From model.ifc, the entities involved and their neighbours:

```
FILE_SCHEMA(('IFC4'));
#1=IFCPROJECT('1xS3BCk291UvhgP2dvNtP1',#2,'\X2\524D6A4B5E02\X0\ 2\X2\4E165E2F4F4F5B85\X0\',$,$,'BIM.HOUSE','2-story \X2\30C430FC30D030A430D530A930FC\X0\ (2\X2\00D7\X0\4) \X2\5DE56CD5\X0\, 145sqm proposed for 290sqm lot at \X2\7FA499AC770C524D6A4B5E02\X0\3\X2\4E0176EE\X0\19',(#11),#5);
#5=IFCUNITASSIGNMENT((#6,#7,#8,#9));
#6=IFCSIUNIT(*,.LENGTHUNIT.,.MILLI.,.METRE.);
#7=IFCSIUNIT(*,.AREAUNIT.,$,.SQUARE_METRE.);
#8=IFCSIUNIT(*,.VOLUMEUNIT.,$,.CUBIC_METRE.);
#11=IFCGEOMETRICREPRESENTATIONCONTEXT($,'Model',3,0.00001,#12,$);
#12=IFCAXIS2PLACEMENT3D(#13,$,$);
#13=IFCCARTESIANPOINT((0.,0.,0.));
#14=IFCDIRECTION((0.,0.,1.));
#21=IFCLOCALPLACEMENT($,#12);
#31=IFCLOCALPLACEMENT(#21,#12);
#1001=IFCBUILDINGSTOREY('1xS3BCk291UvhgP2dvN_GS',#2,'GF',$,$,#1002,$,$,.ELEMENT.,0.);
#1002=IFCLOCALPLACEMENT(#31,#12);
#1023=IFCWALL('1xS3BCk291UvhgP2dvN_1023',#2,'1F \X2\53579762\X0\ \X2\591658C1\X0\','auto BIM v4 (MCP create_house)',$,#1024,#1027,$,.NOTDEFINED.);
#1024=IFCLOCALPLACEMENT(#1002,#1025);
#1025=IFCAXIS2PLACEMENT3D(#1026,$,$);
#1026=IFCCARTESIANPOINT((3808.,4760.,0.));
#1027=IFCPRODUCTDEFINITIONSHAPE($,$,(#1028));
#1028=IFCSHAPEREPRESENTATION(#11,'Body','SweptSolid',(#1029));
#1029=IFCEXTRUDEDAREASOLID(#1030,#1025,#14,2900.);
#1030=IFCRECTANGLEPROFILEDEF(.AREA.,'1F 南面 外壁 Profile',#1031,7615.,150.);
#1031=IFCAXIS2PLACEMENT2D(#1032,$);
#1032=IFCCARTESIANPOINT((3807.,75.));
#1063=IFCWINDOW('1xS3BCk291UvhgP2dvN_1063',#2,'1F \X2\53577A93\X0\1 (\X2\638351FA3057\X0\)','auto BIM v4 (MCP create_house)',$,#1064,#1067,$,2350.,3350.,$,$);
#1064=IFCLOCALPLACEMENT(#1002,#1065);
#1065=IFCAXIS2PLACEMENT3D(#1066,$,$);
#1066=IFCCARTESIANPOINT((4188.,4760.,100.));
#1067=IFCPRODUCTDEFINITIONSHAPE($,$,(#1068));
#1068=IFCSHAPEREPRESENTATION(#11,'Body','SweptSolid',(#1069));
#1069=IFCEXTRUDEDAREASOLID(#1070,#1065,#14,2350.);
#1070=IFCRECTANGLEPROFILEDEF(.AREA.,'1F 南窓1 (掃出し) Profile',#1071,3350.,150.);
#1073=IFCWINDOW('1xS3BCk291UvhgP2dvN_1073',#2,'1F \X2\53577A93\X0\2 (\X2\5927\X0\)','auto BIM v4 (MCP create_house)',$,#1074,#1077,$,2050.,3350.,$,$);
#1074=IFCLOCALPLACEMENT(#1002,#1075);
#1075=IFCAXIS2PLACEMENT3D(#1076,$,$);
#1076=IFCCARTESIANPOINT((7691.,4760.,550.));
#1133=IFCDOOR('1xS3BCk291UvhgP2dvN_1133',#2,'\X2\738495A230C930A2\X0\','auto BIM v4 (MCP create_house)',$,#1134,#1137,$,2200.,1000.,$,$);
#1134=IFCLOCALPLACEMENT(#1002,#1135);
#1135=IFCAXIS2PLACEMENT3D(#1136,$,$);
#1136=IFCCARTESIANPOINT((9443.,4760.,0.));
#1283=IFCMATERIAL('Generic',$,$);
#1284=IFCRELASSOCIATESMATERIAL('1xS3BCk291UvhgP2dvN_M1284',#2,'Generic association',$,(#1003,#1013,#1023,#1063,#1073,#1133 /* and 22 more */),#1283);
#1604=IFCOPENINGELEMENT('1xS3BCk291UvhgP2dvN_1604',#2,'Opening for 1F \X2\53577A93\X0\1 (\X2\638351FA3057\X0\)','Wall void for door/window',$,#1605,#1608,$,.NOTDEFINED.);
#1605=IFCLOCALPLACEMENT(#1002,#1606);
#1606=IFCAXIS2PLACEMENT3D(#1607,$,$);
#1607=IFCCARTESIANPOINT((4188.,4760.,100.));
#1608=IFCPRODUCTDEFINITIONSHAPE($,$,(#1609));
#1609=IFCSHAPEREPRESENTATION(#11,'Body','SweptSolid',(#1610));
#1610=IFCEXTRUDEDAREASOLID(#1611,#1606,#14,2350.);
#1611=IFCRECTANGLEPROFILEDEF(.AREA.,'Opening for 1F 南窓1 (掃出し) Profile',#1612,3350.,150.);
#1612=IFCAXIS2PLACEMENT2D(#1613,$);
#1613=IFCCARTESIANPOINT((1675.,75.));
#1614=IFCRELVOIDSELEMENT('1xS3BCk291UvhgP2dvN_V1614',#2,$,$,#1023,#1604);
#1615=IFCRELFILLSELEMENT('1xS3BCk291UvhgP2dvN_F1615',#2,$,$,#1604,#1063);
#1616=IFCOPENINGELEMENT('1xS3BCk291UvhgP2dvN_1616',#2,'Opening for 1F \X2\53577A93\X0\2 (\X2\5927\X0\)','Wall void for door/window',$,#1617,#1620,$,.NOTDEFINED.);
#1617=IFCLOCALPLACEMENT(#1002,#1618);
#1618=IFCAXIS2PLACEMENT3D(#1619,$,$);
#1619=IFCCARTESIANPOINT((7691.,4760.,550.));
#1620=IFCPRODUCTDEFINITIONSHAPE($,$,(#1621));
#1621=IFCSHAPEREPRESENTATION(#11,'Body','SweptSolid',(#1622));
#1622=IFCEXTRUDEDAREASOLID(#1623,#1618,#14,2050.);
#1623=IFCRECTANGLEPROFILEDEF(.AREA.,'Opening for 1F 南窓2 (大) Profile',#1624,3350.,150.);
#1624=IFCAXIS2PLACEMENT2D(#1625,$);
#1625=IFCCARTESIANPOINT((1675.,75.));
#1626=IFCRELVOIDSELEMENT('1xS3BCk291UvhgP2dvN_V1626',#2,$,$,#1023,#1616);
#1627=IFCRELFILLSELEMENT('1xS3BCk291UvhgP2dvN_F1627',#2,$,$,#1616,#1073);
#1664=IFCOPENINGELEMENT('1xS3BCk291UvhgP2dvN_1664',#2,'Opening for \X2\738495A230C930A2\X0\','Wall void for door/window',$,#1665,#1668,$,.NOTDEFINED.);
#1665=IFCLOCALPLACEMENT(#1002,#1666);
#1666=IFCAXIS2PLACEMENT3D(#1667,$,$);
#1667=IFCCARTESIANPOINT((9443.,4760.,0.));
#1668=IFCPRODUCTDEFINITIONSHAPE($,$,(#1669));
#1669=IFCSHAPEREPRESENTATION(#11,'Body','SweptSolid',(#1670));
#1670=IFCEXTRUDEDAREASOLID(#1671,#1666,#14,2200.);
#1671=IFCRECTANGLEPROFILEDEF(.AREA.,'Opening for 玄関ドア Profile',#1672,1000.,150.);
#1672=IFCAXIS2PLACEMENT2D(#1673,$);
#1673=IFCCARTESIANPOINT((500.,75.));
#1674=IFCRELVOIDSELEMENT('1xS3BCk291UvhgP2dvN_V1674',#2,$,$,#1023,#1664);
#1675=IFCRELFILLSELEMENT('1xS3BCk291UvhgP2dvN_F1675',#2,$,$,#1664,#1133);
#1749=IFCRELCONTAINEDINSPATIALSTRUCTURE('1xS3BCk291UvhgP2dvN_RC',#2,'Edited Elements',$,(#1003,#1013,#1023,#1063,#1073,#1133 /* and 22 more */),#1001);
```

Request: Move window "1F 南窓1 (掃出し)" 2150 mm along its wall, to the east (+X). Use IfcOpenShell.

```python
import ifcopenshell
import ifcopenshell.api.geometry
import ifcopenshell.util.placement

model = ifcopenshell.open("model.ifc")

window = model.by_id(1063)
opening = window.FillsVoids[0].RelatingOpeningElement
wall = opening.VoidsElements[0].RelatingBuildingElement

wall_matrix = ifcopenshell.util.placement.get_local_placement(wall.ObjectPlacement)
shift = wall_matrix[:3, 0] * 2150.0
before = ifcopenshell.util.placement.get_local_placement(window.ObjectPlacement)[:3, 3].copy()

# The window is not placed relative to its opening, so move both.
for product in (opening, window):
    matrix = ifcopenshell.util.placement.get_local_placement(product.ObjectPlacement)
    matrix[:3, 3] += shift
    ifcopenshell.api.geometry.edit_object_placement(model, product=product, matrix=matrix, is_si=False)

after = ifcopenshell.util.placement.get_local_placement(window.ObjectPlacement)[:3, 3]
print("window moved by", (after - before).round(3) + 0.0)

model.write("model_rev.ifc")
```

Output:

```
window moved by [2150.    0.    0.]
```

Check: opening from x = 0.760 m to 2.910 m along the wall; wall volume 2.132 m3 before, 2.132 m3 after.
